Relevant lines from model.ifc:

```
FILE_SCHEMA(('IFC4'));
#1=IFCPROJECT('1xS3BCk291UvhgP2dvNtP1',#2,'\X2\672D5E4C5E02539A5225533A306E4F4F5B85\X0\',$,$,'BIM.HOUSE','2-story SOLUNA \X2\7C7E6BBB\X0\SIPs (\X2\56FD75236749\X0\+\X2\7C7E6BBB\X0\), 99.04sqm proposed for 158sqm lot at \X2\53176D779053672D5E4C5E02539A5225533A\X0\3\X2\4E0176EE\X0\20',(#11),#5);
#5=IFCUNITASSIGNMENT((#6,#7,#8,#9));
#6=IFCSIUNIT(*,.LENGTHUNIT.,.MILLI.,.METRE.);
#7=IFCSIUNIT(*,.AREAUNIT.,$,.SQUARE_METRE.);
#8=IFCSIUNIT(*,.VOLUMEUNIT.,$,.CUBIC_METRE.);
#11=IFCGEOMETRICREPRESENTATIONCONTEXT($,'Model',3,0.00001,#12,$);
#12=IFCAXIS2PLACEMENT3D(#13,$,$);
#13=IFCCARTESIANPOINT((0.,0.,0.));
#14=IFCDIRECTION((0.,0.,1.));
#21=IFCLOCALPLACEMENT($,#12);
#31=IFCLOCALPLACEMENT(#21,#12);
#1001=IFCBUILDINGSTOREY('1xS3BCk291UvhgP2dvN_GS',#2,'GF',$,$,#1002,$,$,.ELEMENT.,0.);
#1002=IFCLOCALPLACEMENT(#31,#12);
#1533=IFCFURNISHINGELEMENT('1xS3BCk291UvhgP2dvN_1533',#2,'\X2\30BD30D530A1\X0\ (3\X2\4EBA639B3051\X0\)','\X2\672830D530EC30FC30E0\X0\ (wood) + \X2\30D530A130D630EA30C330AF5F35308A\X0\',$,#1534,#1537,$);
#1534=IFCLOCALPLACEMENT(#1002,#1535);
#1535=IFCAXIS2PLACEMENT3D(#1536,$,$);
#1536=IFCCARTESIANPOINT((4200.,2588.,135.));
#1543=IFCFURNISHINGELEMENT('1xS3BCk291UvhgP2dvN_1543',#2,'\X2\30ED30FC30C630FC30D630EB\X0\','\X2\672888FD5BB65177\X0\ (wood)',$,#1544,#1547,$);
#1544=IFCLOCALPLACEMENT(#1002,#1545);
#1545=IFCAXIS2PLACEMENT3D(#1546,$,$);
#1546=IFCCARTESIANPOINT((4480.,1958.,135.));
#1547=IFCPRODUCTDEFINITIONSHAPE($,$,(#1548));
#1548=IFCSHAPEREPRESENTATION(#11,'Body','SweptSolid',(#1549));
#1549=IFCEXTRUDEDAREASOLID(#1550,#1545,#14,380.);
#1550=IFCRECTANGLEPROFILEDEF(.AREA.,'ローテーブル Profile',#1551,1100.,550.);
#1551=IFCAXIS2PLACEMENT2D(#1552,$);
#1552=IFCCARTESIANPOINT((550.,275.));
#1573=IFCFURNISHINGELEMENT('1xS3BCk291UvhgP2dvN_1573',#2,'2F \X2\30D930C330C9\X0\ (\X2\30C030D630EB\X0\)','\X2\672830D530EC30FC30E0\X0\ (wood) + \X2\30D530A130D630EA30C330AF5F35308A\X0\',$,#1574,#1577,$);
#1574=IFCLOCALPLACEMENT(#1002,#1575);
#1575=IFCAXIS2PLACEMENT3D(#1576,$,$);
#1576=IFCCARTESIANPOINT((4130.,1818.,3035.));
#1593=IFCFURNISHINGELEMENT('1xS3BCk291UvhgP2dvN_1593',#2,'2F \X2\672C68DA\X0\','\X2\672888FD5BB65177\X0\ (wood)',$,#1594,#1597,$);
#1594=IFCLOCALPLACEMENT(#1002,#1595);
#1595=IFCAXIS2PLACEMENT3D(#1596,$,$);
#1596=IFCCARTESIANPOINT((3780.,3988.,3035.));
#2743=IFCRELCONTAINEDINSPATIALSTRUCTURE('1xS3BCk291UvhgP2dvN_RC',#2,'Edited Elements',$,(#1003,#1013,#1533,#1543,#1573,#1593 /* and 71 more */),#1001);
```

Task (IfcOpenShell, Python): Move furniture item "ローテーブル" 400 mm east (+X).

```python
import ifcopenshell
import ifcopenshell.api.geometry
import ifcopenshell.util.placement
import ifcopenshell.util.unit

model = ifcopenshell.open("model.ifc")
unit_scale = ifcopenshell.util.unit.calculate_unit_scale(model)

item = model.by_guid("1xS3BCk291UvhgP2dvN_1543")
matrix = ifcopenshell.util.placement.get_local_placement(item.ObjectPlacement)
matrix[0, 3] += 0.4 / unit_scale
ifcopenshell.api.geometry.edit_object_placement(model, product=item, matrix=matrix, is_si=False)

print(ifcopenshell.util.placement.get_local_placement(item.ObjectPlacement).round(3) + 0.0)

model.write("model_updated.ifc")
```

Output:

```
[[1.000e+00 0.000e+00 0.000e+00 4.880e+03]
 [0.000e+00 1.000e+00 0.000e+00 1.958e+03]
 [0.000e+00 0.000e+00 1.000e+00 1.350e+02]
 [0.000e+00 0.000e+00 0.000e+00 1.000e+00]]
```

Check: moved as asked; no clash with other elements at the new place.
